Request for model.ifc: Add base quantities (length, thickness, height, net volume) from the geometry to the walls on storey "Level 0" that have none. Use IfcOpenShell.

First a look at what the model holds.

```python
import ifcopenshell
import ifcopenshell.util.element
import ifcopenshell.util.unit

model = ifcopenshell.open("model.ifc")
print(model.schema)
for unit_type in ("LENGTHUNIT", "AREAUNIT", "VOLUMEUNIT"):
    print(unit_type, ifcopenshell.util.unit.calculate_unit_scale(model, unit_type))
storey = next(s for s in model.by_type("IfcBuildingStorey") if s.Name == "Level 0")
walls = [e for e in ifcopenshell.util.element.get_decomposition(storey) if e.is_a("IfcWall")]
for e in sorted(walls, key=lambda e: e.id()):
    print(e.id(), e.is_a(), e.Name, list(ifcopenshell.util.element.get_psets(e, qtos_only=True)), sep=" | ")
```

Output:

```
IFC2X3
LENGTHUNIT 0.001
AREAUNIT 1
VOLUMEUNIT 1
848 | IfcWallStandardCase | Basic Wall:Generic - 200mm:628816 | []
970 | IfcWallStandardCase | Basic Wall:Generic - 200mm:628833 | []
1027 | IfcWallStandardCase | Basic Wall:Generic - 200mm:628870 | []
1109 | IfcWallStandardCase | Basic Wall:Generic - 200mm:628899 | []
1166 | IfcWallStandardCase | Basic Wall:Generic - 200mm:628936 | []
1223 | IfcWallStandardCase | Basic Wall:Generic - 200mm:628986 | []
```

```python
import ifcopenshell
import ifcopenshell.api.pset
import ifcopenshell.geom
import ifcopenshell.util.element
import ifcopenshell.util.shape
import ifcopenshell.util.unit

model = ifcopenshell.open("model.ifc")
unit_scale = ifcopenshell.util.unit.calculate_unit_scale(model)
volume_scale = ifcopenshell.util.unit.calculate_unit_scale(model, "VOLUMEUNIT")
settings = ifcopenshell.geom.settings()

storey = next(s for s in model.by_type("IfcBuildingStorey") if s.Name == "Level 0")
walls = [e for e in ifcopenshell.util.element.get_decomposition(storey) if e.is_a("IfcWall")]

for e in sorted(walls, key=lambda e: e.id()):
    if ifcopenshell.util.element.get_psets(e, qtos_only=True, should_inherit=False):
        continue
    # Geometry comes back in metres, in the element's own axes.
    shape = ifcopenshell.geom.create_shape(settings, e)
    values = {
        "Length": ifcopenshell.util.shape.get_x(shape.geometry) / unit_scale,
        "Width": ifcopenshell.util.shape.get_y(shape.geometry) / unit_scale,
        "Height": ifcopenshell.util.shape.get_z(shape.geometry) / unit_scale,
        "NetVolume": ifcopenshell.util.shape.get_volume(shape.geometry) / volume_scale,
    }
    qto = ifcopenshell.api.pset.add_qto(model, product=e, name="BaseQuantities")
    ifcopenshell.api.pset.edit_qto(model, qto=qto, properties=values)
    print(e.id(), {k: round(v, 3) for k, v in values.items()})

model.write("model_edited.ifc")
```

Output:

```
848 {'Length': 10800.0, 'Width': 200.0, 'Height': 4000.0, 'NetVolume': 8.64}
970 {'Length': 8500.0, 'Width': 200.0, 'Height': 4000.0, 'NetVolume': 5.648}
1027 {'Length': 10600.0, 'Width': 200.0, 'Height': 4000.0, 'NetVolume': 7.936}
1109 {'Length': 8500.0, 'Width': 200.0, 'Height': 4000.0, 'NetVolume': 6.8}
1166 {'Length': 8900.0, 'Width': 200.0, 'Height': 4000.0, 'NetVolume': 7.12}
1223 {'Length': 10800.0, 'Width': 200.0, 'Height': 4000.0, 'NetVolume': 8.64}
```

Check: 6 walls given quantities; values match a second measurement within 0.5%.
